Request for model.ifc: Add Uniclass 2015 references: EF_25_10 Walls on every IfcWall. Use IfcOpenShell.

First a look at what the model holds.

```python
import ifcopenshell

model = ifcopenshell.open("model.ifc")
print(model.schema)
print("classifications:", [c.Name for c in model.by_type("IfcClassification")])
for ifc_class in ("IfcDoor", "IfcRoof", "IfcStair", "IfcWall", "IfcWindow"):
    print(ifc_class, len(model.by_type(ifc_class)))
```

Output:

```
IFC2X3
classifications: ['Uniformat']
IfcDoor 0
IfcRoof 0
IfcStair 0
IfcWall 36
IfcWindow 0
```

```python
import ifcopenshell
import ifcopenshell.api.classification

model = ifcopenshell.open("model.ifc")

# IFC2X3 requires Source and Edition and has no link from the project to the system.
system = model.create_entity("IfcClassification", Source="NBS", Edition="2015", Name="Uniclass 2015")

codes = {
    "IfcWall": ("EF_25_10", "Walls"),
}
for ifc_class, (code, name) in codes.items():
    products = model.by_type(ifc_class)
    ifcopenshell.api.classification.add_reference(
        model, products=products, classification=system, identification=code, name=name
    )
    print(code, len(products))

model.write("model-out.ifc")
```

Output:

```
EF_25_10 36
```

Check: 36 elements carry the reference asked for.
